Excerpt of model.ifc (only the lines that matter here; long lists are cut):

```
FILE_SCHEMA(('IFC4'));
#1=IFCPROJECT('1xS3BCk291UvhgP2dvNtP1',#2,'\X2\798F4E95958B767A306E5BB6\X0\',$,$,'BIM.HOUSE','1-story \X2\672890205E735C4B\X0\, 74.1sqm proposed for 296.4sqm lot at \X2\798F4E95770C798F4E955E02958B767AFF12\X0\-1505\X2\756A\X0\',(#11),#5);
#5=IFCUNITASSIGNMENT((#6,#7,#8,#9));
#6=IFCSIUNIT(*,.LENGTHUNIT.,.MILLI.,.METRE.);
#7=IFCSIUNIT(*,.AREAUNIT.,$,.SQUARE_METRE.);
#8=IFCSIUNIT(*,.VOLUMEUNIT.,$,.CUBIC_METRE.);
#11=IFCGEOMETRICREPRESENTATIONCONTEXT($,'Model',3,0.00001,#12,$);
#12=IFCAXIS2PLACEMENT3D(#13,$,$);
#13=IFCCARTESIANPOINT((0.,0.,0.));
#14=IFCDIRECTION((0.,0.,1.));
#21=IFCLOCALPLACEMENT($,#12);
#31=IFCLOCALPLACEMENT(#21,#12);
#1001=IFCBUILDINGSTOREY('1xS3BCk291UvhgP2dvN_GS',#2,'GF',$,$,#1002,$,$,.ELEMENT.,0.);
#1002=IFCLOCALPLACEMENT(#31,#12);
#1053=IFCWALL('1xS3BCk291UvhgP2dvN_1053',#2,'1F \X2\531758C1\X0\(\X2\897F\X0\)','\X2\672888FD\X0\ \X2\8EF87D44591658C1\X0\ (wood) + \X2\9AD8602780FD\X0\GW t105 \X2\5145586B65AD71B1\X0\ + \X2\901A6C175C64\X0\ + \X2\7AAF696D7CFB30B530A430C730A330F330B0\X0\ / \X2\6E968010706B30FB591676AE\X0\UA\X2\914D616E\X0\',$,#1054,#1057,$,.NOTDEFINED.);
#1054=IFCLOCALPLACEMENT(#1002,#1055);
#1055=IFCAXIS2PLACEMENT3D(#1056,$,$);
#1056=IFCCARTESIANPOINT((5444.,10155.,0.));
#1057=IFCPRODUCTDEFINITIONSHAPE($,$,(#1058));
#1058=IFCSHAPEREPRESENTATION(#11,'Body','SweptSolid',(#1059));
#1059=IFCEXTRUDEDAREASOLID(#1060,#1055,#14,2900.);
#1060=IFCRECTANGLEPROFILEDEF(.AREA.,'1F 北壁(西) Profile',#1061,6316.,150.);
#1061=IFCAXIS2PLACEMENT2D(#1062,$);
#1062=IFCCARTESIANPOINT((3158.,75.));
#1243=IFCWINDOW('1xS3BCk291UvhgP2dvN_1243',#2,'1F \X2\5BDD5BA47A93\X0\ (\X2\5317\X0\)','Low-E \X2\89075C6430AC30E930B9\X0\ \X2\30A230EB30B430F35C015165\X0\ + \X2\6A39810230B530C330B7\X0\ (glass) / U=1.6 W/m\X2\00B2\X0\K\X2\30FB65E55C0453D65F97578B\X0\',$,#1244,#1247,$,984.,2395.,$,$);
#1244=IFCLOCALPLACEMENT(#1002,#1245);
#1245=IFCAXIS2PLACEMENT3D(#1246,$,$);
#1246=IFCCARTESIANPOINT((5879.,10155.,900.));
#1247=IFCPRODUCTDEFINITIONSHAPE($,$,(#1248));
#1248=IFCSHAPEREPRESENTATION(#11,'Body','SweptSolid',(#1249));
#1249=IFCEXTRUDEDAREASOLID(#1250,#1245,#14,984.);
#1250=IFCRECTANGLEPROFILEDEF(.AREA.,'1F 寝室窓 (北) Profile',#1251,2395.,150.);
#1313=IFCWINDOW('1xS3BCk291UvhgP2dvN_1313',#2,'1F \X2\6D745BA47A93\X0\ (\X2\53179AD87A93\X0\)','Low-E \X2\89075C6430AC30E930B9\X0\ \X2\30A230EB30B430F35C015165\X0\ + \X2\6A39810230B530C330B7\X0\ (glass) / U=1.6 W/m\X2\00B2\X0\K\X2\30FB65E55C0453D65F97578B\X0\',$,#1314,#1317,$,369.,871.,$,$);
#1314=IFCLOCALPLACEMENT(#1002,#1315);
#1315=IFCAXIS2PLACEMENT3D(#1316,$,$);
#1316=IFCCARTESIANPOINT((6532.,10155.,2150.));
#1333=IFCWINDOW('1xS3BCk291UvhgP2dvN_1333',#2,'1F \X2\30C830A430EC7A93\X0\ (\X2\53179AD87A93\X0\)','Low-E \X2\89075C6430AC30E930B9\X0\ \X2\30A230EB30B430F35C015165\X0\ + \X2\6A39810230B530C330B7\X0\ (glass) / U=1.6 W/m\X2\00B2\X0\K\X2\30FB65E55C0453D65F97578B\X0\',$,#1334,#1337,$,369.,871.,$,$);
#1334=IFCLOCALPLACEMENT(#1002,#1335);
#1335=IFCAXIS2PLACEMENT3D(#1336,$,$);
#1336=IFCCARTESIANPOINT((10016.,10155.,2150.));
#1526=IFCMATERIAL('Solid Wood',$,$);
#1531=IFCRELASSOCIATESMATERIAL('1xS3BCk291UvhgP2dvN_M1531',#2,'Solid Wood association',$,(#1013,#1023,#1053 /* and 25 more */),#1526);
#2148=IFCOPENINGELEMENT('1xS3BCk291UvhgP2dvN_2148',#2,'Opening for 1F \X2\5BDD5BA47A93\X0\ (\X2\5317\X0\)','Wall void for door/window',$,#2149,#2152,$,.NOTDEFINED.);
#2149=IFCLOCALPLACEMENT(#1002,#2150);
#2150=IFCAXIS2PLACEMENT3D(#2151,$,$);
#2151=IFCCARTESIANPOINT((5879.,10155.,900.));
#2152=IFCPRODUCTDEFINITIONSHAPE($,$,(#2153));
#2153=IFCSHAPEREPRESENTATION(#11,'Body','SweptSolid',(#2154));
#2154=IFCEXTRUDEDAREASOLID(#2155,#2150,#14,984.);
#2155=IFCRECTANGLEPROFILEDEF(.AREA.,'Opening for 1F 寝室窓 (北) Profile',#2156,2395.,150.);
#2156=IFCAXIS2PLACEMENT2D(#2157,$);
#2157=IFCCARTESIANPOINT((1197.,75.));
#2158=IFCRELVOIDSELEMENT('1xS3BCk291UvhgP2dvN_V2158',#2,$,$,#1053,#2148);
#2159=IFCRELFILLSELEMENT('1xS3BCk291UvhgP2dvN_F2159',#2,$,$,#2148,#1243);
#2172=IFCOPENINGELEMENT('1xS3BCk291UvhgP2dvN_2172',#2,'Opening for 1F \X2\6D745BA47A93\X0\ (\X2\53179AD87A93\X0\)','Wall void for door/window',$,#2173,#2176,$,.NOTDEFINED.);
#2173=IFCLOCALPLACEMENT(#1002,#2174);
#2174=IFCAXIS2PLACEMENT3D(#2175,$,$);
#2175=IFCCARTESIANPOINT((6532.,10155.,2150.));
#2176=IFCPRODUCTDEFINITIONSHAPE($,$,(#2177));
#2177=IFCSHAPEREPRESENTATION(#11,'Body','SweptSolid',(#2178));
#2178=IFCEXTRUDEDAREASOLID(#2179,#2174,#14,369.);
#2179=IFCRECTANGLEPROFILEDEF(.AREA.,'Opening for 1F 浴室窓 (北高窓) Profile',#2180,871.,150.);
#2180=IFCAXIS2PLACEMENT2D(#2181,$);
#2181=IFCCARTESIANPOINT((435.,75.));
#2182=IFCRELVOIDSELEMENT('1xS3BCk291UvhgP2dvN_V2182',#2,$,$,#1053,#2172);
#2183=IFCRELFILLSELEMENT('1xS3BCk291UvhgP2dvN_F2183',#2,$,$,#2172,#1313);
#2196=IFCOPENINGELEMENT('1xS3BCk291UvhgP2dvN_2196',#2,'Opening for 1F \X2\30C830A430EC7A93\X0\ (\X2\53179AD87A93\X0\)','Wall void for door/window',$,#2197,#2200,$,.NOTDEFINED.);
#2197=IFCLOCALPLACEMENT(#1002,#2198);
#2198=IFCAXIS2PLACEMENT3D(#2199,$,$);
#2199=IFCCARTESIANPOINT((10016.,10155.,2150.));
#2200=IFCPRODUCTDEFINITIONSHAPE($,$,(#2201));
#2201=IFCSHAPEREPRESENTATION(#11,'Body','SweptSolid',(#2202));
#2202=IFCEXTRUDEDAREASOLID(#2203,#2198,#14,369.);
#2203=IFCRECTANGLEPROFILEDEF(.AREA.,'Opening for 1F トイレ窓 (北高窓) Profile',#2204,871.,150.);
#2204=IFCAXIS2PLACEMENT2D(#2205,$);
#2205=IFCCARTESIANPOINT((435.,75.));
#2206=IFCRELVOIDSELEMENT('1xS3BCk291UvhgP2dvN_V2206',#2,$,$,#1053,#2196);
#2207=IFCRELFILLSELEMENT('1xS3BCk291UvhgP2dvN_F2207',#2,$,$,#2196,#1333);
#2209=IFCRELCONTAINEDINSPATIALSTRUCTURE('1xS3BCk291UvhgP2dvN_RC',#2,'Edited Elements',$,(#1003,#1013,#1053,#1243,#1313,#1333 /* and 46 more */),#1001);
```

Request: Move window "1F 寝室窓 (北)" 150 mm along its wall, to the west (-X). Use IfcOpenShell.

```python
import ifcopenshell
import ifcopenshell.api.geometry
import ifcopenshell.util.placement

model = ifcopenshell.open("model.ifc")

window = model.by_guid("1xS3BCk291UvhgP2dvN_1243")
opening = window.FillsVoids[0].RelatingOpeningElement
wall = opening.VoidsElements[0].RelatingBuildingElement

wall_matrix = ifcopenshell.util.placement.get_local_placement(wall.ObjectPlacement)
shift = wall_matrix[:3, 0] * -150.0
before = ifcopenshell.util.placement.get_local_placement(window.ObjectPlacement)[:3, 3].copy()

# The window is not placed relative to its opening, so move both.
for product in (opening, window):
    matrix = ifcopenshell.util.placement.get_local_placement(product.ObjectPlacement)
    matrix[:3, 3] += shift
    ifcopenshell.api.geometry.edit_object_placement(model, product=product, matrix=matrix, is_si=False)

after = ifcopenshell.util.placement.get_local_placement(window.ObjectPlacement)[:3, 3]
print("window moved by", (after - before).round(3) + 0.0)

model.write("model_v2.ifc")
```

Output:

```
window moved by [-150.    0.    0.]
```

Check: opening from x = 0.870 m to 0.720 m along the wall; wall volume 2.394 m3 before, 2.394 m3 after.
